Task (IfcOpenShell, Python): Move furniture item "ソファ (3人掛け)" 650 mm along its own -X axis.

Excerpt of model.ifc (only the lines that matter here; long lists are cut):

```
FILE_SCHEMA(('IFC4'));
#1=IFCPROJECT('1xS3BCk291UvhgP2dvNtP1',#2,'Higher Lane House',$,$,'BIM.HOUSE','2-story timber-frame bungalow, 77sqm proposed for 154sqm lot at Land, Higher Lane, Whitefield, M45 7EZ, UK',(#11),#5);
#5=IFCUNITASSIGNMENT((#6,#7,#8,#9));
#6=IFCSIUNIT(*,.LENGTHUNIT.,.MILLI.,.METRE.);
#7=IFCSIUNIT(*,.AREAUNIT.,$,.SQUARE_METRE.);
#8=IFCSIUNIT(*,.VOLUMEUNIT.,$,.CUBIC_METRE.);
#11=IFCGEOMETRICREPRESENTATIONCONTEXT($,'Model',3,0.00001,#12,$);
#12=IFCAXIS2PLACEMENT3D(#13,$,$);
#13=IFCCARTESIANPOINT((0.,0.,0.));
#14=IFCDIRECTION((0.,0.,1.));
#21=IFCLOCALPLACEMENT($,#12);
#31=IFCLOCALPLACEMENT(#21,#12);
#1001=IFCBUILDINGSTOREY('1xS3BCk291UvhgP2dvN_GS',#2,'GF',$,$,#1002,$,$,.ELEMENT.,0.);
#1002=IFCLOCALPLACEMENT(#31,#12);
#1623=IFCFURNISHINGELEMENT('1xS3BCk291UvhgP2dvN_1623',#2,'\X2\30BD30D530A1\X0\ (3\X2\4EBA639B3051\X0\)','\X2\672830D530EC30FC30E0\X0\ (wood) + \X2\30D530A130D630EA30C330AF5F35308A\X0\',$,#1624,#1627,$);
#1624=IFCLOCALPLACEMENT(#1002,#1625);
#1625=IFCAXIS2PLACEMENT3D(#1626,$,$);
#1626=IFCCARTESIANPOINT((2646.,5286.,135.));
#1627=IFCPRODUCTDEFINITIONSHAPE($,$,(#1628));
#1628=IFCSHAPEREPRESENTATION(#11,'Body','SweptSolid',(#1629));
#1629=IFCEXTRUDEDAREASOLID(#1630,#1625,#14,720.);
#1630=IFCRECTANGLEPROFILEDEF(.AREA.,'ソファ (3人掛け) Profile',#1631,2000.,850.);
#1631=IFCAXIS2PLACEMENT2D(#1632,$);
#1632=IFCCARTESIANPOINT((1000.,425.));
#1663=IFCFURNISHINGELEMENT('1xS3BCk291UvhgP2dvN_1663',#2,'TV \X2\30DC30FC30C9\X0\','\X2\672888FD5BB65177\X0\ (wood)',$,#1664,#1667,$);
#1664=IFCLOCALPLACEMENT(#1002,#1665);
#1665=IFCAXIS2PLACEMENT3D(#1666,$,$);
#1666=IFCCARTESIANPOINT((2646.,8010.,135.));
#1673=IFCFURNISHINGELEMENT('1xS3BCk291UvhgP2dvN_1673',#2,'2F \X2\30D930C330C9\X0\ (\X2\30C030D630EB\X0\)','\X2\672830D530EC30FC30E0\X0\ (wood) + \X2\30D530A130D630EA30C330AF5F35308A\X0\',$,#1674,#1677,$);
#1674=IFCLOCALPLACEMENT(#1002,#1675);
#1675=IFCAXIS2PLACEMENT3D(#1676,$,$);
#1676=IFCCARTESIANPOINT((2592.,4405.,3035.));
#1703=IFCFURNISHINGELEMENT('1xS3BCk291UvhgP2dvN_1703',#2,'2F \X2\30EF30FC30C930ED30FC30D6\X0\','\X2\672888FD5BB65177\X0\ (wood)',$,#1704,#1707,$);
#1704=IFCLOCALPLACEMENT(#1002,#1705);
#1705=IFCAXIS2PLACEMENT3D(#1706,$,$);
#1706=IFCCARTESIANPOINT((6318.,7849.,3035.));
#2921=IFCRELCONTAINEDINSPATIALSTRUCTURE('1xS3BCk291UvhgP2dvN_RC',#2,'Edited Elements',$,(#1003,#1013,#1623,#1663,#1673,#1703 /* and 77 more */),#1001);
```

```python
import ifcopenshell
import ifcopenshell.api.geometry
import ifcopenshell.util.placement
import ifcopenshell.util.unit

model = ifcopenshell.open("model.ifc")
unit_scale = ifcopenshell.util.unit.calculate_unit_scale(model)

item = model.by_id(1623)
matrix = ifcopenshell.util.placement.get_local_placement(item.ObjectPlacement)
matrix[:3, 3] -= matrix[:3, 0] * 0.65 / unit_scale
ifcopenshell.api.geometry.edit_object_placement(model, product=item, matrix=matrix, is_si=False)

print(ifcopenshell.util.placement.get_local_placement(item.ObjectPlacement).round(3) + 0.0)

model.write("model-out.ifc")
```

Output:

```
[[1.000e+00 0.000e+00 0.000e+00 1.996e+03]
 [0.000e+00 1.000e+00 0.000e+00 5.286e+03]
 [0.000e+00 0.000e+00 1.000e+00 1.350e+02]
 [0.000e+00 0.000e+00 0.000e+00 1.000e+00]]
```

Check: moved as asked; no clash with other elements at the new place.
